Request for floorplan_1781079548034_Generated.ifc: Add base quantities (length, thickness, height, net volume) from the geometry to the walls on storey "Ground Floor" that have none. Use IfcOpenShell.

First a look at what the model holds.

```python
import ifcopenshell
import ifcopenshell.util.element
import ifcopenshell.util.unit

model = ifcopenshell.open("floorplan_1781079548034_Generated.ifc")
print(model.schema)
for unit_type in ("LENGTHUNIT", "AREAUNIT", "VOLUMEUNIT"):
    print(unit_type, ifcopenshell.util.unit.calculate_unit_scale(model, unit_type))
storey = next(s for s in model.by_type("IfcBuildingStorey") if s.Name == "Ground Floor")
walls = [e for e in ifcopenshell.util.element.get_decomposition(storey) if e.is_a("IfcWall")]
for e in sorted(walls, key=lambda e: e.id()):
    print(e.id(), e.is_a(), e.Name, list(ifcopenshell.util.element.get_psets(e, qtos_only=True)), sep=" | ")
```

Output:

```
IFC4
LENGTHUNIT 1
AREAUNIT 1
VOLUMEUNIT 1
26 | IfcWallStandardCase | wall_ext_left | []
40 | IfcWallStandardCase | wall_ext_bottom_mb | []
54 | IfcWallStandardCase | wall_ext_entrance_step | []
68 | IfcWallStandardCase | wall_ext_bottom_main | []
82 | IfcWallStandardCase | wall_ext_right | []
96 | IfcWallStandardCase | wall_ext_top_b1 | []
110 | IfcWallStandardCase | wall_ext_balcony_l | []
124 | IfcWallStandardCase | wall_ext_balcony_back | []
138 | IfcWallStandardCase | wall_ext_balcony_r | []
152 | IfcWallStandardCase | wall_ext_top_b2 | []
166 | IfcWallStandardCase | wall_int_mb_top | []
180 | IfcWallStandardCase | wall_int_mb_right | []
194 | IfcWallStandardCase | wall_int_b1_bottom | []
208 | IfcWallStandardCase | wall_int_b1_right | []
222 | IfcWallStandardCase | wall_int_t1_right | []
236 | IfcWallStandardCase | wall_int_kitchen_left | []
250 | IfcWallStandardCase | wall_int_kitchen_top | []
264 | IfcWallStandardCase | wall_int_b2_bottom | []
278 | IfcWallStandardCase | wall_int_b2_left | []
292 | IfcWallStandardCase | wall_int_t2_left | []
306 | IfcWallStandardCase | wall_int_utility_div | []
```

```python
import ifcopenshell
import ifcopenshell.api.pset
import ifcopenshell.geom
import ifcopenshell.util.element
import ifcopenshell.util.shape
import ifcopenshell.util.unit

model = ifcopenshell.open("floorplan_1781079548034_Generated.ifc")
unit_scale = ifcopenshell.util.unit.calculate_unit_scale(model)
volume_scale = ifcopenshell.util.unit.calculate_unit_scale(model, "VOLUMEUNIT")
settings = ifcopenshell.geom.settings()

storey = next(s for s in model.by_type("IfcBuildingStorey") if s.Name == "Ground Floor")
walls = [e for e in ifcopenshell.util.element.get_decomposition(storey) if e.is_a("IfcWall")]

for e in sorted(walls, key=lambda e: e.id()):
    if ifcopenshell.util.element.get_psets(e, qtos_only=True, should_inherit=False):
        continue
    # Geometry comes back in metres, in the element's own axes.
    shape = ifcopenshell.geom.create_shape(settings, e)
    values = {
        "Length": ifcopenshell.util.shape.get_x(shape.geometry) / unit_scale,
        "Width": ifcopenshell.util.shape.get_y(shape.geometry) / unit_scale,
        "Height": ifcopenshell.util.shape.get_z(shape.geometry) / unit_scale,
        "NetVolume": ifcopenshell.util.shape.get_volume(shape.geometry) / volume_scale,
    }
    qto = ifcopenshell.api.pset.add_qto(model, product=e, name="Qto_WallBaseQuantities")
    ifcopenshell.api.pset.edit_qto(model, qto=qto, properties=values)
    print(e.id(), {k: round(v, 3) for k, v in values.items()})

model.write("floorplan_1781079548034_Generated_v2.ifc")
```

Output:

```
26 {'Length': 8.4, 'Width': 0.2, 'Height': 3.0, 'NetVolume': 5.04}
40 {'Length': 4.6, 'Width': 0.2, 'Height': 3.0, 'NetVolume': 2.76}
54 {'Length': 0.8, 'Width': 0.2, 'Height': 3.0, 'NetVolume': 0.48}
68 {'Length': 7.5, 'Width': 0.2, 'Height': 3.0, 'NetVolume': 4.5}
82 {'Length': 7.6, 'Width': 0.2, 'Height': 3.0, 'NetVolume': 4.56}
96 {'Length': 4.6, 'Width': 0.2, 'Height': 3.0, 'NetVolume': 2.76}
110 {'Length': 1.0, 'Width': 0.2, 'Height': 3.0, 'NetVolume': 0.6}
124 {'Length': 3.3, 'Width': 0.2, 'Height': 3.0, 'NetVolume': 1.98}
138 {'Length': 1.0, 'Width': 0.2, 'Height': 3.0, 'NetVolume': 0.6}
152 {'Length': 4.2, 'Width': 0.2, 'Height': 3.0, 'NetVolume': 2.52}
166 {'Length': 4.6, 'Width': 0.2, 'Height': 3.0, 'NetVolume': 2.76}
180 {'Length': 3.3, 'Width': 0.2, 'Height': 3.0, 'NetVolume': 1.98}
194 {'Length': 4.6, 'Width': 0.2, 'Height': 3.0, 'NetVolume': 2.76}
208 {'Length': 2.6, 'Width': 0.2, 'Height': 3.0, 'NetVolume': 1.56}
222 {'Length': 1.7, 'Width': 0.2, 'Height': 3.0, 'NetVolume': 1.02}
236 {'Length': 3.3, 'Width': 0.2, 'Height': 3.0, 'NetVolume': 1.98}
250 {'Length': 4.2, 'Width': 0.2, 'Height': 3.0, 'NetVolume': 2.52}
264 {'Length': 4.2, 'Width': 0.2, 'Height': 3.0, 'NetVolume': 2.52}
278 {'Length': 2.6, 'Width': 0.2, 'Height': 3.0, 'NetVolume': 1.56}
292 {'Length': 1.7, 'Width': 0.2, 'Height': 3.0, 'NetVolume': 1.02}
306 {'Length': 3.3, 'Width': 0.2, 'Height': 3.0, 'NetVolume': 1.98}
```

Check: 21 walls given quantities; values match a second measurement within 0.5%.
